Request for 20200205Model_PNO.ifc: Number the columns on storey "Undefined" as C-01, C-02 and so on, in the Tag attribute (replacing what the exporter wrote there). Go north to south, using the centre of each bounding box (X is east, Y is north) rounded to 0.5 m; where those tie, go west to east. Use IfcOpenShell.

First a look at what the model holds.

```python
import ifcopenshell
import ifcopenshell.util.element
import ifcopenshell.util.placement

model = ifcopenshell.open("20200205Model_PNO.ifc")
print(model.schema)
storey = next(s for s in model.by_type("IfcBuildingStorey") if s.Name == "Undefined")
columns = [e for e in ifcopenshell.util.element.get_decomposition(storey) if e.is_a("IfcColumn")]
for e in sorted(columns, key=lambda e: e.id()):
    origin = ifcopenshell.util.placement.get_local_placement(e.ObjectPlacement)[:3, 3]
    print(e.id(), e.Tag, e.Name, origin.round(2) + 0.0, sep=" | ")
```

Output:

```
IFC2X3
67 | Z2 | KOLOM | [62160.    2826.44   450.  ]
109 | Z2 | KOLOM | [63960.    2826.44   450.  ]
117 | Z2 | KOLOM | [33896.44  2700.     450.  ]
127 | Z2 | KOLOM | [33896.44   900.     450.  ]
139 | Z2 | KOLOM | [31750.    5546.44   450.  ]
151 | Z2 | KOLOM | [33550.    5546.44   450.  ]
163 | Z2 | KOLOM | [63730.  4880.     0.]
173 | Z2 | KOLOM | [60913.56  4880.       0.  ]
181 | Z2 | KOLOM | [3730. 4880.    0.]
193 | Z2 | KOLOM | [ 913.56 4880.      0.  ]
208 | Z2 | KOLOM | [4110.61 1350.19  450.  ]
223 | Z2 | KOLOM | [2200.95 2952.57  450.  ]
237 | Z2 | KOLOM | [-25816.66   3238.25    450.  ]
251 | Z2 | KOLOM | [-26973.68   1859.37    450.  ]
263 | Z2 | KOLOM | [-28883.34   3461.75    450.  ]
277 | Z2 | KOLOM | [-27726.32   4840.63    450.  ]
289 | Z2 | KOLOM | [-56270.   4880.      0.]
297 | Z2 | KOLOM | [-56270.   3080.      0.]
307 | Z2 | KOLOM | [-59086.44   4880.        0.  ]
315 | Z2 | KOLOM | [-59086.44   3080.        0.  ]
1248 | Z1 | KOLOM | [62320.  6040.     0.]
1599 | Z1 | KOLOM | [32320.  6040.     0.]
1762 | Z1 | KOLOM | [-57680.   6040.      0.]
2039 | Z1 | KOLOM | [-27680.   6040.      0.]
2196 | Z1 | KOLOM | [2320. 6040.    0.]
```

```python
import ifcopenshell
import ifcopenshell.geom
import ifcopenshell.util.element
import ifcopenshell.util.shape

model = ifcopenshell.open("20200205Model_PNO.ifc")
settings = ifcopenshell.geom.settings()
settings.set("use-world-coords", True)


def centre(element):
    shape = ifcopenshell.geom.create_shape(settings, element)
    return ifcopenshell.util.shape.get_bbox_centroid(shape.geometry)


storey = next(s for s in model.by_type("IfcBuildingStorey") if s.Name == "Undefined")
columns = [e for e in ifcopenshell.util.element.get_decomposition(storey) if e.is_a("IfcColumn")]

# Insertion points can sit at a corner or the storey origin, so sort by the geometry (in metres).
centres = {e: centre(e) for e in columns}
columns.sort(key=lambda e: (-round(centres[e][1] / 0.5), centres[e][0]))

for i, e in enumerate(columns, start=1):
    number = f"C-{i:02d}"
    e.Tag = number
    print(e.id(), number)

model.write("20200205Model_PNO_v2.ifc")
```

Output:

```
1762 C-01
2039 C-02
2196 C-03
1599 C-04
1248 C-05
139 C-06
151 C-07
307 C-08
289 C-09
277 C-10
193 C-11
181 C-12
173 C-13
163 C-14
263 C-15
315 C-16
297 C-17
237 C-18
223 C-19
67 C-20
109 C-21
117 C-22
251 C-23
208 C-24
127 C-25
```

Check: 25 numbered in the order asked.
